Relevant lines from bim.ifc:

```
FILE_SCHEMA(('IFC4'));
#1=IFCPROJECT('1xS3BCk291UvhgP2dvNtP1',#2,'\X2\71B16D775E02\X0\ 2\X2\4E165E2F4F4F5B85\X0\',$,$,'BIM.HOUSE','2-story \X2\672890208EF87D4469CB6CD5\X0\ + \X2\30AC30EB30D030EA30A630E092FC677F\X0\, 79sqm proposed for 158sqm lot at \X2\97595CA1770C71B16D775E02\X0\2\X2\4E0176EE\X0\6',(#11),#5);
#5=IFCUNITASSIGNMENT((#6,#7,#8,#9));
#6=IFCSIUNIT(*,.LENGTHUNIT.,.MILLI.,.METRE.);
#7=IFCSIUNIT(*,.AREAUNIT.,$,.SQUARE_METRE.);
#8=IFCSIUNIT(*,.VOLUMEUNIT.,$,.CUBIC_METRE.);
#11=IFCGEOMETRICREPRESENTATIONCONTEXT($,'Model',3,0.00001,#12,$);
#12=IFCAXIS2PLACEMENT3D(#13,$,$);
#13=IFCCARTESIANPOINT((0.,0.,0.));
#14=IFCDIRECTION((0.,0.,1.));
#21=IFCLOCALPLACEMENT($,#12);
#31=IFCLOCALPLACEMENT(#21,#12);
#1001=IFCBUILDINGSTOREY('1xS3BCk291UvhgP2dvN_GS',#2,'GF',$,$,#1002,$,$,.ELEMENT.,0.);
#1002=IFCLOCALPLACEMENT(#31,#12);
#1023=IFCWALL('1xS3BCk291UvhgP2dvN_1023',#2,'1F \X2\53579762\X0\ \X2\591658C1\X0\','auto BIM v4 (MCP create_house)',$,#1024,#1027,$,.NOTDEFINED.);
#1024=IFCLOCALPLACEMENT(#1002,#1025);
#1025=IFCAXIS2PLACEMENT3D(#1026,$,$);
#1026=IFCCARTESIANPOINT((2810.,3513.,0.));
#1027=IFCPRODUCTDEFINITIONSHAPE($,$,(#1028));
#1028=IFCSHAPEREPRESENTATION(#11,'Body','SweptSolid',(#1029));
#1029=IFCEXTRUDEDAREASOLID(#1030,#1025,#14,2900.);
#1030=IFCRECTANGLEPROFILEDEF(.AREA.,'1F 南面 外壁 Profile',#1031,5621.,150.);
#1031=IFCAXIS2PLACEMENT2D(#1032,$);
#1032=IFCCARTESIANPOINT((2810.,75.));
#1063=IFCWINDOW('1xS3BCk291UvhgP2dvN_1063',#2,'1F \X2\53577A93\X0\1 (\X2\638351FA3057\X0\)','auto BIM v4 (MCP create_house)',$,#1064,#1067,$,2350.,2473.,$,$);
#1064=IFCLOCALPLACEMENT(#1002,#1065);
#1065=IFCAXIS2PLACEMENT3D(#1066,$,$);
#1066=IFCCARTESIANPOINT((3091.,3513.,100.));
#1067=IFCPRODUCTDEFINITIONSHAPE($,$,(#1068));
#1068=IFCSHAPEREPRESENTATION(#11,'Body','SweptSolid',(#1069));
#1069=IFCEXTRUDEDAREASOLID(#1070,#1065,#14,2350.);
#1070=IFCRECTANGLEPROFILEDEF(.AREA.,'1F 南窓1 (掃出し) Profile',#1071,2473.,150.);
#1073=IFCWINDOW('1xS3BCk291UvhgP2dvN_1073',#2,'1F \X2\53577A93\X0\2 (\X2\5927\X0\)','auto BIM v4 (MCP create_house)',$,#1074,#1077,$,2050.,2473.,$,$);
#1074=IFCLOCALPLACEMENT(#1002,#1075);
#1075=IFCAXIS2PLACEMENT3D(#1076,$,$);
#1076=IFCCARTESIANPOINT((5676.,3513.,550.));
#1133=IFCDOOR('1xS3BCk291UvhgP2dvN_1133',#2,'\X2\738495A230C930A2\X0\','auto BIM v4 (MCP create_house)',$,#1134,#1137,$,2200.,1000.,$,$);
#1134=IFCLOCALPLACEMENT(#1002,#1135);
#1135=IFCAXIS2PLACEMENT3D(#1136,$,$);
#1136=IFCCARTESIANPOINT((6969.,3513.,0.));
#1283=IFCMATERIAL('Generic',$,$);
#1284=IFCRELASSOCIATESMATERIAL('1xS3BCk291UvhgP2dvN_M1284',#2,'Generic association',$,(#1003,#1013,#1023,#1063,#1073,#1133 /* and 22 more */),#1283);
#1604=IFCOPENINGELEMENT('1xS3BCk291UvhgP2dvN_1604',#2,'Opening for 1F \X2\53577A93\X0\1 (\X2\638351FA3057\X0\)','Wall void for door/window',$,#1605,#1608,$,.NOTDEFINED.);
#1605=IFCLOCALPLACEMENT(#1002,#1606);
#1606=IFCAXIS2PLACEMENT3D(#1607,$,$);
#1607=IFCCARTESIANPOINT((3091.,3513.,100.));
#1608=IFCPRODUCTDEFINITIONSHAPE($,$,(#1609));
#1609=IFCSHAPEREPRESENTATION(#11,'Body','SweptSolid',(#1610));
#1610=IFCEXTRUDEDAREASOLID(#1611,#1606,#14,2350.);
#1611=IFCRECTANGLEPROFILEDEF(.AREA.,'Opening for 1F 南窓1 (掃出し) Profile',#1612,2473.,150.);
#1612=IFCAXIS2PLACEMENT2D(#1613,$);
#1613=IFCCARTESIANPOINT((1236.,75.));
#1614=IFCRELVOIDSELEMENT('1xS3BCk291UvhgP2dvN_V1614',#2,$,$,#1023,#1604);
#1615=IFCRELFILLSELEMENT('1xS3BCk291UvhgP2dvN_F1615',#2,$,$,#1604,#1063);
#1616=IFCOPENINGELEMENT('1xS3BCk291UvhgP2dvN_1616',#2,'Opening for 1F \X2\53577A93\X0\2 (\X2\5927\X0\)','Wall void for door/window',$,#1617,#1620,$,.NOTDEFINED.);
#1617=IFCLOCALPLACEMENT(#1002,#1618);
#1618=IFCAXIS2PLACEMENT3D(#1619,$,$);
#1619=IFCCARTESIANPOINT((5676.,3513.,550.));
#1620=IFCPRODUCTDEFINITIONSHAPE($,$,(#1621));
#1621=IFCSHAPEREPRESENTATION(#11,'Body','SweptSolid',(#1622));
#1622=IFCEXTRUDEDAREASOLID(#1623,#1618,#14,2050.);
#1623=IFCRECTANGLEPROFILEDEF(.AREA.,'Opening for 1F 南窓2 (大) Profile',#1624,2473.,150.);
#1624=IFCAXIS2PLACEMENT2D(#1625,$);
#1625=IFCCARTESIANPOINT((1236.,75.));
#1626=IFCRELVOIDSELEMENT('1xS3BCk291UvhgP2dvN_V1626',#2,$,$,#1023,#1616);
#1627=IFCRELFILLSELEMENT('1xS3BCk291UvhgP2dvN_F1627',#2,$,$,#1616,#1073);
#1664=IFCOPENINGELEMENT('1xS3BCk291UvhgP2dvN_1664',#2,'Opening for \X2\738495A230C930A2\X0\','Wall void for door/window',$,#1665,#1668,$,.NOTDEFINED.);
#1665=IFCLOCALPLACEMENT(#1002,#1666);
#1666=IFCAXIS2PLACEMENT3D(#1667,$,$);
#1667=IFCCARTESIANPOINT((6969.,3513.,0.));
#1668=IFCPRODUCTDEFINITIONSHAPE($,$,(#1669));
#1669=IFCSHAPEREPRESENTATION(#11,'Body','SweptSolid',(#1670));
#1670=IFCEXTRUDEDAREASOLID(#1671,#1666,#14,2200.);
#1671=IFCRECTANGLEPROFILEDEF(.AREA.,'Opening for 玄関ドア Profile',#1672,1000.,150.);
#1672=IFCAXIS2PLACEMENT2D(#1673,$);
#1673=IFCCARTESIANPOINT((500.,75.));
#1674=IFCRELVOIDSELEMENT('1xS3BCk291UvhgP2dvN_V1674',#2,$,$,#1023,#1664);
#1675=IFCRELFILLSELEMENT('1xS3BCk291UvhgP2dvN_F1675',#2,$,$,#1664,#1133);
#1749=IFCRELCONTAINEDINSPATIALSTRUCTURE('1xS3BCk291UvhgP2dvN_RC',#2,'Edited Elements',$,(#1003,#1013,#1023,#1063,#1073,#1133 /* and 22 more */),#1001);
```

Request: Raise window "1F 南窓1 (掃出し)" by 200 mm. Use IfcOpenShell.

```python
import numpy as np
import ifcopenshell
import ifcopenshell.api.geometry
import ifcopenshell.util.placement
import ifcopenshell.util.unit

model = ifcopenshell.open("bim.ifc")
unit_scale = ifcopenshell.util.unit.calculate_unit_scale(model)

window = model.by_guid("1xS3BCk291UvhgP2dvN_1063")
opening = window.FillsVoids[0].RelatingOpeningElement
dz = 200.0

shift = np.array([0.0, 0.0, dz])
# The window is not placed relative to its opening, so move both.
for product in (opening, window):
    matrix = ifcopenshell.util.placement.get_local_placement(product.ObjectPlacement)
    matrix[:3, 3] += shift
    ifcopenshell.api.geometry.edit_object_placement(model, product=product, matrix=matrix, is_si=False)

print(f"moved by {dz * unit_scale:+.3f} m")

model.write("bim-out.ifc")
```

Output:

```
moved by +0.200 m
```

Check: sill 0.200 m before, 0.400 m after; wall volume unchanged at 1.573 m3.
